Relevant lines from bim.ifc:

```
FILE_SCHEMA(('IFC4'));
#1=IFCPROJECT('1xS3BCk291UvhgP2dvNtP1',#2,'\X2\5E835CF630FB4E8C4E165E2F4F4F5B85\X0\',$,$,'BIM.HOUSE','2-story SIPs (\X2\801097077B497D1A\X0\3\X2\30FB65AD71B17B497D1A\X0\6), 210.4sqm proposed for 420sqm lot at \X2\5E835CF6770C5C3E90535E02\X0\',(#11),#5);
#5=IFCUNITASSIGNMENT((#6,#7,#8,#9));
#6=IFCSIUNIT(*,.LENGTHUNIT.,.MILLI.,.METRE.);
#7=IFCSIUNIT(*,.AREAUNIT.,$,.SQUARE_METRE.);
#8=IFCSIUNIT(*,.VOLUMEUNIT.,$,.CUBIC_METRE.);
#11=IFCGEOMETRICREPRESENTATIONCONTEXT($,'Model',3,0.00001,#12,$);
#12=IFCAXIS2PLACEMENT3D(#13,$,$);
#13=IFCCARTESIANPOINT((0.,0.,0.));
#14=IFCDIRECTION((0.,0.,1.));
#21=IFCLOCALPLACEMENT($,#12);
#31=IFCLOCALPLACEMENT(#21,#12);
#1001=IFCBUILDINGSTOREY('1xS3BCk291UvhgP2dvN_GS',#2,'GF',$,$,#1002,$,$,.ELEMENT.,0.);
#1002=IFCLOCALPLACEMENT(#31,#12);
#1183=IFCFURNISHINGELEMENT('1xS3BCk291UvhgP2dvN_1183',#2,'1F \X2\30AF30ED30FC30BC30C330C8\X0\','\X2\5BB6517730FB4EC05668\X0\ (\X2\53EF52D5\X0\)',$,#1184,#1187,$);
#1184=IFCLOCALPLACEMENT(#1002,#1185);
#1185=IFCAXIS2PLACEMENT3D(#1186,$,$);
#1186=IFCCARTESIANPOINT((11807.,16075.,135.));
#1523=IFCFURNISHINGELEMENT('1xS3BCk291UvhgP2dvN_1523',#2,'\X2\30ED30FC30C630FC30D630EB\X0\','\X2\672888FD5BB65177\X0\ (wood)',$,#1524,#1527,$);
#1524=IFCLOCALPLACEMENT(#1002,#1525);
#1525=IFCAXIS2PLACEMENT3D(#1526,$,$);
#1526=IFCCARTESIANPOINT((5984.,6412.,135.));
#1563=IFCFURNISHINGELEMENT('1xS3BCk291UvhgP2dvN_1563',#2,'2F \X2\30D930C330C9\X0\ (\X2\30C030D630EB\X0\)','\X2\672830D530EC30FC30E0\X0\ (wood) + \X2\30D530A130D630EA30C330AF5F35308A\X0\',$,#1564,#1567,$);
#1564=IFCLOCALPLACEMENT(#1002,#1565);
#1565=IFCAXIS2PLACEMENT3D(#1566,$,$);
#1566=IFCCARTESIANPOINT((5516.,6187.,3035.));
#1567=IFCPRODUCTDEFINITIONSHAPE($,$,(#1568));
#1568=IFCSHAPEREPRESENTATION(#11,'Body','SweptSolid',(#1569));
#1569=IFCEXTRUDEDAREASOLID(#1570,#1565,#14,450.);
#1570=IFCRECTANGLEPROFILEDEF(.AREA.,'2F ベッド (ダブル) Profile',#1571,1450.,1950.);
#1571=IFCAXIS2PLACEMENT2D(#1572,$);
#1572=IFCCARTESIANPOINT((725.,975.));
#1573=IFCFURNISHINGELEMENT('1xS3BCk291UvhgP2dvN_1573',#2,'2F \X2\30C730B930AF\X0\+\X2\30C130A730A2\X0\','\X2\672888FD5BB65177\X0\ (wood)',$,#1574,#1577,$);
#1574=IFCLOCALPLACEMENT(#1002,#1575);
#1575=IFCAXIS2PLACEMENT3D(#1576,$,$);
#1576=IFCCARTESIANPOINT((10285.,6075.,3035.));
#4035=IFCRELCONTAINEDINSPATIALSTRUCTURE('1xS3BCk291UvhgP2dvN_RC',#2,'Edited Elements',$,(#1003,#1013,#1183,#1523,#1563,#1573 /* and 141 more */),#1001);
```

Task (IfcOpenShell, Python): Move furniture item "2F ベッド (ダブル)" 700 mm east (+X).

```python
import ifcopenshell
import ifcopenshell.api.geometry
import ifcopenshell.util.placement
import ifcopenshell.util.unit

model = ifcopenshell.open("bim.ifc")
unit_scale = ifcopenshell.util.unit.calculate_unit_scale(model)

item = model.by_guid("1xS3BCk291UvhgP2dvN_1563")
matrix = ifcopenshell.util.placement.get_local_placement(item.ObjectPlacement)
matrix[0, 3] += 0.7 / unit_scale
ifcopenshell.api.geometry.edit_object_placement(model, product=item, matrix=matrix, is_si=False)

print(ifcopenshell.util.placement.get_local_placement(item.ObjectPlacement).round(3) + 0.0)

model.write("bim_edited.ifc")
```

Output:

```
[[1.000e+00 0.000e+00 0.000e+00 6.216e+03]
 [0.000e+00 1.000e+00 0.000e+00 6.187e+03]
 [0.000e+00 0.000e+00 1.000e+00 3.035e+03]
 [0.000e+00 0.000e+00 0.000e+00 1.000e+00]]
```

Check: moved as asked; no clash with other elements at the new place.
